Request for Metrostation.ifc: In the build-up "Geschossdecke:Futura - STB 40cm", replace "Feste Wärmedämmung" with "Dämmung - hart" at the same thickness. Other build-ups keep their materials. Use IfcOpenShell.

First a look at what the model holds.

```python
import ifcopenshell
import ifcopenshell.util.element

model = ifcopenshell.open("Metrostation.ifc")
print(model.schema)
for layer_set in model.by_type("IfcMaterialLayerSet"):
    if layer_set.LayerSetName == "Geschossdecke:Futura - STB 40cm":
        for layer in layer_set.MaterialLayers:
            print(layer.id(), layer.Material and layer.Material.Name, layer.LayerThickness, sep=" | ")
        print(len(ifcopenshell.util.element.get_elements_by_material(model, layer_set)), "elements and types use it")
print(sorted(m.Name for m in model.by_type("IfcMaterial") if m.Name)[:60])
```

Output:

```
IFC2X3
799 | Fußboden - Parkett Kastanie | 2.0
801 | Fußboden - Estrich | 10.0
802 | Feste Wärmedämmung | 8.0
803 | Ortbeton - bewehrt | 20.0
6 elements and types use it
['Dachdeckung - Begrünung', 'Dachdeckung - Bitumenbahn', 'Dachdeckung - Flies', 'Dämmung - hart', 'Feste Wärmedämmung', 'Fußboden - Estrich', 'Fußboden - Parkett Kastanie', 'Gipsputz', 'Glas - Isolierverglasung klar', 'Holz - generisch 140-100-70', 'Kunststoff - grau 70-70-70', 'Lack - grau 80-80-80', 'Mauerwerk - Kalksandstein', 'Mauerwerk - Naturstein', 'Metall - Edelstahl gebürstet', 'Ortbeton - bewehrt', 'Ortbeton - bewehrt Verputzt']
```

```python
import ifcopenshell
import ifcopenshell.api.material

model = ifcopenshell.open("Metrostation.ifc")

layer_set = next(s for s in model.by_type("IfcMaterialLayerSet") if s.LayerSetName == "Geschossdecke:Futura - STB 40cm")
layer = next(l for l in layer_set.MaterialLayers if l.Material and l.Material.Name == "Feste Wärmedämmung")
material = next(m for m in model.by_type("IfcMaterial") if m.Name == "Dämmung - hart")

# Point this one layer at the other material; renaming the old one would change it everywhere.
ifcopenshell.api.material.edit_layer(model, layer=layer, attributes={}, material=material)

print([l.Material.Name if l.Material else None for l in layer_set.MaterialLayers])

model.write("Metrostation_v2.ifc")
```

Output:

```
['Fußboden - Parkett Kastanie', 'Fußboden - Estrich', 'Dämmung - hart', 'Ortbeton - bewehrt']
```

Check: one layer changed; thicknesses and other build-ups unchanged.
